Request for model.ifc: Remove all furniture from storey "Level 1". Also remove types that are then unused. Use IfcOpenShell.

First a look at what the model holds.

```python
import ifcopenshell
import ifcopenshell.util.element

model = ifcopenshell.open("model.ifc")
print(model.schema)
storey = next(s for s in model.by_type("IfcBuildingStorey") if s.Name == "Level 1")
furniture = [e for e in ifcopenshell.util.element.get_decomposition(storey) if e.is_a("IfcFurnishingElement")]
seen = {}
for e in furniture:
    element_type = ifcopenshell.util.element.get_type(e)
    name = element_type.Name if element_type not in (None, e) else None
    seen[name] = seen.get(name, 0) + 1
for name, count in sorted(seen.items(), key=str):
    print(count, "x", name)
```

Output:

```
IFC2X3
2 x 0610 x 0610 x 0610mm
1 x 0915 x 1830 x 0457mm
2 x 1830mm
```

```python
import ifcopenshell
import ifcopenshell.api.root
import ifcopenshell.util.element

model = ifcopenshell.open("model.ifc")

storey = next(s for s in model.by_type("IfcBuildingStorey") if s.Name == "Level 1")
furniture = [e for e in ifcopenshell.util.element.get_decomposition(storey) if e.is_a("IfcFurnishingElement")]
types = {ifcopenshell.util.element.get_type(e) for e in furniture} - {None, *furniture}

for e in furniture:
    ifcopenshell.api.root.remove_product(model, product=e)
print(len(furniture), "removed")

unused = [t for t in types if not ifcopenshell.util.element.get_types(t)]
for t in unused:
    ifcopenshell.api.root.remove_product(model, product=t)
print(len(unused), "unused types removed")

model.write("model-out.ifc")
```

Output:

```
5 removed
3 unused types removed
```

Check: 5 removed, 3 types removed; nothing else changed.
